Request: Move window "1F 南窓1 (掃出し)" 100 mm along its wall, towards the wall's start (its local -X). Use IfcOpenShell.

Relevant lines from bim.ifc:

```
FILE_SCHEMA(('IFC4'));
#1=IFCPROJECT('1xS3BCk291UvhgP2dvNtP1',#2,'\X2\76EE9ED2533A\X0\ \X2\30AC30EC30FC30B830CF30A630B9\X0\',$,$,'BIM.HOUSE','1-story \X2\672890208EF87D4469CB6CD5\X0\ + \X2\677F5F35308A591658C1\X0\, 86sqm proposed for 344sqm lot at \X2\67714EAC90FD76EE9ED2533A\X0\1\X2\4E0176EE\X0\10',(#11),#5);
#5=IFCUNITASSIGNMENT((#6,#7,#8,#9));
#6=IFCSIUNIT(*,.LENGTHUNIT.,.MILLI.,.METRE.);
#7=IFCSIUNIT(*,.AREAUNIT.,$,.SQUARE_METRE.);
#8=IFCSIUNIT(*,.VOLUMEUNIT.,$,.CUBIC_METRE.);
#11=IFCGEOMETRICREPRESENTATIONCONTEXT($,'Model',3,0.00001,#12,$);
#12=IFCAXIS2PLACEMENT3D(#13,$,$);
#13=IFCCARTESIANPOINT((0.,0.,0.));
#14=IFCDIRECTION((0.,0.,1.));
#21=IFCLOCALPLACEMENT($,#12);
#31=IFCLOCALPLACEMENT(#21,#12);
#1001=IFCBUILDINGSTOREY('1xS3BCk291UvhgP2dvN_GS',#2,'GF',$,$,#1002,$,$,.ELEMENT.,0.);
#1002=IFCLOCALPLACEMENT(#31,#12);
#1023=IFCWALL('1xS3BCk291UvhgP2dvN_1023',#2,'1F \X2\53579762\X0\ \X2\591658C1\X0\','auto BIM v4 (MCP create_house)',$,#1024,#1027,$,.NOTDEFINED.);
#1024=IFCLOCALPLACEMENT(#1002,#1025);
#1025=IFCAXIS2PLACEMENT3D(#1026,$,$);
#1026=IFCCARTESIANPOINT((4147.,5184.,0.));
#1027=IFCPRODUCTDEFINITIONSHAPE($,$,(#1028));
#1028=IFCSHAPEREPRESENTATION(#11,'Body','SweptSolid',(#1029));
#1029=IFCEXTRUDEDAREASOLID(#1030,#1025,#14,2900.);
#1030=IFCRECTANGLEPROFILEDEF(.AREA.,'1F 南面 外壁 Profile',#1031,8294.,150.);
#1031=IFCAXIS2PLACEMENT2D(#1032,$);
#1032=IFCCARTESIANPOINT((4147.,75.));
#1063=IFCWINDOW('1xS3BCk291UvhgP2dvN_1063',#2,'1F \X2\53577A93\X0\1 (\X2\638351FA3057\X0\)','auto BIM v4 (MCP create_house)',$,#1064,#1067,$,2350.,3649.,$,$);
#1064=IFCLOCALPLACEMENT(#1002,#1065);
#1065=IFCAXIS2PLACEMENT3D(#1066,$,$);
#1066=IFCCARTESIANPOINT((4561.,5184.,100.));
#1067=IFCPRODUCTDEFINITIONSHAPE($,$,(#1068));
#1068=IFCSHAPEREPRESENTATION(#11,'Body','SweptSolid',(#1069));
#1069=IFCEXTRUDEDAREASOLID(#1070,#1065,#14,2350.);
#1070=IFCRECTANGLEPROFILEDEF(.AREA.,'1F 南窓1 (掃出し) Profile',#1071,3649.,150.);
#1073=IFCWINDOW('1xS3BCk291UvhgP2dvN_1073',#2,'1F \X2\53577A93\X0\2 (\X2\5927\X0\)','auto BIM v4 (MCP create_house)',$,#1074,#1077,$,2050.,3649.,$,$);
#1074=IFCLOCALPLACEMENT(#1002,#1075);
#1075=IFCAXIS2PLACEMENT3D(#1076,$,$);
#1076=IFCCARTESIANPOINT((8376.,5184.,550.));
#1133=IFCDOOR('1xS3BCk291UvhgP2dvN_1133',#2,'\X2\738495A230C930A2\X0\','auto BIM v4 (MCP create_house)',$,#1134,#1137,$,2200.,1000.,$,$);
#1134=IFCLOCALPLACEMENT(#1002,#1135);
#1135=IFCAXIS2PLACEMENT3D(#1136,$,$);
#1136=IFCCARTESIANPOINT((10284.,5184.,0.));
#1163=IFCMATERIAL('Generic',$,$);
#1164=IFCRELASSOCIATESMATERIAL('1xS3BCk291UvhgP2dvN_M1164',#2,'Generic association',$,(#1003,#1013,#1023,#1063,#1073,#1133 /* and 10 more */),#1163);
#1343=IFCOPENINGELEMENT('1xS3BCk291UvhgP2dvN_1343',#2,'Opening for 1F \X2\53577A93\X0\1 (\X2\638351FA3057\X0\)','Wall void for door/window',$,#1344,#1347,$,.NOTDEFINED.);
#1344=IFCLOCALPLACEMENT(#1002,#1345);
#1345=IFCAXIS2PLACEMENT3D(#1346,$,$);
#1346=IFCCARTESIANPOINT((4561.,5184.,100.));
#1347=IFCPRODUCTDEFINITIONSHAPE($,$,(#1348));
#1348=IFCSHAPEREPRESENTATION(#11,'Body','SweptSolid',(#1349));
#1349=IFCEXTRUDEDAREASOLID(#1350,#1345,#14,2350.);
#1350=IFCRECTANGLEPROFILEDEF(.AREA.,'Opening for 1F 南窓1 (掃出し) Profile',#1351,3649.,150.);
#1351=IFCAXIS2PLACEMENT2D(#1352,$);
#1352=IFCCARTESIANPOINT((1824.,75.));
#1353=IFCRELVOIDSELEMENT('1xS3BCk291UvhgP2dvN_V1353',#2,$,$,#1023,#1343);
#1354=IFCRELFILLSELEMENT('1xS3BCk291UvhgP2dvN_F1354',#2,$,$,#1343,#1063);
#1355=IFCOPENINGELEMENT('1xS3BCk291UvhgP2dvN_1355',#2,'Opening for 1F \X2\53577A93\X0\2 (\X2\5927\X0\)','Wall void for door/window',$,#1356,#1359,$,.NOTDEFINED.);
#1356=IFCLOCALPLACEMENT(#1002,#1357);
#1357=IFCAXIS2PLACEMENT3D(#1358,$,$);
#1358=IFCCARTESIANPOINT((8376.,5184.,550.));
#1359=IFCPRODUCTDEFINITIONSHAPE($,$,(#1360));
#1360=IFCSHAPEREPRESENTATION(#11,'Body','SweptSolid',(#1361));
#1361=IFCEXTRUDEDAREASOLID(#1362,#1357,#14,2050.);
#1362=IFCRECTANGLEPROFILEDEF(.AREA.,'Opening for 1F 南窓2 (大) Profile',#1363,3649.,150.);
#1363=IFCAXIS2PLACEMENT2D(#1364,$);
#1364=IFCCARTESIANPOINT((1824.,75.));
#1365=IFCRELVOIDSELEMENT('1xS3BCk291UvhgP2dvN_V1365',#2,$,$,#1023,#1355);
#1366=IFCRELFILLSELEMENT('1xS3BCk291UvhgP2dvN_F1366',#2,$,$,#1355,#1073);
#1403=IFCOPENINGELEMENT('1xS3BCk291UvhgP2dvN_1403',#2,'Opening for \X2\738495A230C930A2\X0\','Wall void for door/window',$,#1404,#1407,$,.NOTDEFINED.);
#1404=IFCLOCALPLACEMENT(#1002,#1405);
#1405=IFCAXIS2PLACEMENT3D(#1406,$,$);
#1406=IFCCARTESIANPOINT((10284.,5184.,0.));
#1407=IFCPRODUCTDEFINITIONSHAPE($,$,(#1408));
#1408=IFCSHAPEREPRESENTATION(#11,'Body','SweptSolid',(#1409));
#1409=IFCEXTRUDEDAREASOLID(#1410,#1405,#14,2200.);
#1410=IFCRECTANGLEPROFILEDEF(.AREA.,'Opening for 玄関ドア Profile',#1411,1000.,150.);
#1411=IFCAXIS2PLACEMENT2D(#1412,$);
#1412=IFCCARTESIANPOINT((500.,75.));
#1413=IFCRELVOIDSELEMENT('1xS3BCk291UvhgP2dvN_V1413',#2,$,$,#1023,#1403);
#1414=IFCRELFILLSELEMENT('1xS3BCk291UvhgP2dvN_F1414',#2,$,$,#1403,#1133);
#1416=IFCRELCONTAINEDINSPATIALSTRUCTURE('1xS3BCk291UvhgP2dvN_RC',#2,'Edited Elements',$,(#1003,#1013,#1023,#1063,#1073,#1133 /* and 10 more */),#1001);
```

```python
import ifcopenshell
import ifcopenshell.api.geometry
import ifcopenshell.util.placement
import ifcopenshell.util.unit

model = ifcopenshell.open("bim.ifc")
unit_scale = ifcopenshell.util.unit.calculate_unit_scale(model)

window = model.by_guid("1xS3BCk291UvhgP2dvN_1063")
opening = window.FillsVoids[0].RelatingOpeningElement
wall = opening.VoidsElements[0].RelatingBuildingElement

wall_matrix = ifcopenshell.util.placement.get_local_placement(wall.ObjectPlacement)
shift = wall_matrix[:3, 0] * -0.1 / unit_scale
before = ifcopenshell.util.placement.get_local_placement(window.ObjectPlacement)[:3, 3].copy()

# The window is not placed relative to its opening, so move both.
for product in (opening, window):
    matrix = ifcopenshell.util.placement.get_local_placement(product.ObjectPlacement)
    matrix[:3, 3] += shift
    ifcopenshell.api.geometry.edit_object_placement(model, product=product, matrix=matrix, is_si=False)

after = ifcopenshell.util.placement.get_local_placement(window.ObjectPlacement)[:3, 3]
print("window moved by", (after - before).round(3) + 0.0)

model.write("bim_v2.ifc")
```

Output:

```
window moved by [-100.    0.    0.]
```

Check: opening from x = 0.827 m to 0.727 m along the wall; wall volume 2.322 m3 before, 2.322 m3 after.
